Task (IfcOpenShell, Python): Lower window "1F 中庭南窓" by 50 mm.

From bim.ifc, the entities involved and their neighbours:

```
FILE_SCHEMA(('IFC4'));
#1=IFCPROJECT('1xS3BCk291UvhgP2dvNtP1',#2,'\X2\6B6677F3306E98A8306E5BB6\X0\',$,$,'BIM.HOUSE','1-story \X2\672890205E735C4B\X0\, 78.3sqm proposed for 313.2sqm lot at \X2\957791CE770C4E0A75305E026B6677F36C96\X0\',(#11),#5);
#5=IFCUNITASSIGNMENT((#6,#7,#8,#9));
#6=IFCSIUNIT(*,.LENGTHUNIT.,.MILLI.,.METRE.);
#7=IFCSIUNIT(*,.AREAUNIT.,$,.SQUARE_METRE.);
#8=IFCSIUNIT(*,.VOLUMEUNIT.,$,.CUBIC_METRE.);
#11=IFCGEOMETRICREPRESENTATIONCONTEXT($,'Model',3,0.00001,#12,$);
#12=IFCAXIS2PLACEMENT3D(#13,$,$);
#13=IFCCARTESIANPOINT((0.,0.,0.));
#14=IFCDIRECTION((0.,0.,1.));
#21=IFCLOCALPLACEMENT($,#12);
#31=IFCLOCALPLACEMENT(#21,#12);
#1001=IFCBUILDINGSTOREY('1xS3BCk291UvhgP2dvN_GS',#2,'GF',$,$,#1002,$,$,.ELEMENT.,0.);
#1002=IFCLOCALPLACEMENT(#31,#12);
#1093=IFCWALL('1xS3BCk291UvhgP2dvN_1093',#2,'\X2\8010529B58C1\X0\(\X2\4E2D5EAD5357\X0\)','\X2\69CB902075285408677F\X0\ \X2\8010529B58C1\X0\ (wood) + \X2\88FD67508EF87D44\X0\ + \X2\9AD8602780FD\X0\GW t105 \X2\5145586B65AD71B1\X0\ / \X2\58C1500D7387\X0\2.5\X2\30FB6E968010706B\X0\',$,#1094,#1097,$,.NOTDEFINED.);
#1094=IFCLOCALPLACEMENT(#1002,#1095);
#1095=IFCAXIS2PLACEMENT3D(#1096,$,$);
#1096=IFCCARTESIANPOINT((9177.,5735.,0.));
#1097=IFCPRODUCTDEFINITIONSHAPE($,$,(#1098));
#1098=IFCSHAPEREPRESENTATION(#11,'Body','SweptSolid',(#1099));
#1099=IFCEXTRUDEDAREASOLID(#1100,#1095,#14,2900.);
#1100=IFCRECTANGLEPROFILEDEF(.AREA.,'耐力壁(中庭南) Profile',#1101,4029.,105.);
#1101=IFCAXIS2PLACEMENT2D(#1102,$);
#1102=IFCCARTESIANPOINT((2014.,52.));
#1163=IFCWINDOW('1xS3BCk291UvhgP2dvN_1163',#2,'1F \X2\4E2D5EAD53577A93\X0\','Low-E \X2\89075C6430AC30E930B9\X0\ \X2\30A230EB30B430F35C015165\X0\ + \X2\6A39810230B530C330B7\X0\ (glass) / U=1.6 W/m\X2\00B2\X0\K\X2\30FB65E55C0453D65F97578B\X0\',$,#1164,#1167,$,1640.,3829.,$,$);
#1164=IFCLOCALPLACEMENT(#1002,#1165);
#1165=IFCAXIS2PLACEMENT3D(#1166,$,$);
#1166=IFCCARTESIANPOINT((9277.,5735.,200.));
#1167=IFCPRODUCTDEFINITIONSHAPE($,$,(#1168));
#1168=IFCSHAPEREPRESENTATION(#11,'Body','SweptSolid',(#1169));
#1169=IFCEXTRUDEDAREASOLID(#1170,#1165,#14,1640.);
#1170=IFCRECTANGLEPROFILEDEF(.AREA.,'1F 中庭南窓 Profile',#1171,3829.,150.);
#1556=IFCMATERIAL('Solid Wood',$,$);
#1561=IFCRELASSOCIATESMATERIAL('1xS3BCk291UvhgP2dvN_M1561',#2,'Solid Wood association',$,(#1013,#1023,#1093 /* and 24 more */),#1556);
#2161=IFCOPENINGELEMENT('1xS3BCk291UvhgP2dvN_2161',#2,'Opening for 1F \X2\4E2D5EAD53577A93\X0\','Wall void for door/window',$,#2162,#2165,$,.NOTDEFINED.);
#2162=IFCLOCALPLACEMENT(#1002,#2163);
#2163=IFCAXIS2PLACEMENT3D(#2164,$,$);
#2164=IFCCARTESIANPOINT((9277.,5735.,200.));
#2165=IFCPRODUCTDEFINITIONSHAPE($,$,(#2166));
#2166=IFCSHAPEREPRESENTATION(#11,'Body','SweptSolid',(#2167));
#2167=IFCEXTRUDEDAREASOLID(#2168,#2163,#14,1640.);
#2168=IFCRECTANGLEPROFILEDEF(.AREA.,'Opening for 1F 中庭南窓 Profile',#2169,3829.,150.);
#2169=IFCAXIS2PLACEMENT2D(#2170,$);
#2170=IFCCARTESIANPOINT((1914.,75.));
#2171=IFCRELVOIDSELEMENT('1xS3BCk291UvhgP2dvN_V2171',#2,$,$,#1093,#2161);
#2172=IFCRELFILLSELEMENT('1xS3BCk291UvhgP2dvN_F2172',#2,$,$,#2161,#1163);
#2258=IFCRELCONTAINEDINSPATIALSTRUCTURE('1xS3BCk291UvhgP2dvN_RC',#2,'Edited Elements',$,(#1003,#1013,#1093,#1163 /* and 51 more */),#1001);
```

```python
import numpy as np
import ifcopenshell
import ifcopenshell.api.geometry
import ifcopenshell.util.placement
import ifcopenshell.util.unit

model = ifcopenshell.open("bim.ifc")
unit_scale = ifcopenshell.util.unit.calculate_unit_scale(model)

window = model.by_id(1163)
opening = window.FillsVoids[0].RelatingOpeningElement
dz = -50.0

shift = np.array([0.0, 0.0, dz])
# The window is not placed relative to its opening, so move both.
for product in (opening, window):
    matrix = ifcopenshell.util.placement.get_local_placement(product.ObjectPlacement)
    matrix[:3, 3] += shift
    ifcopenshell.api.geometry.edit_object_placement(model, product=product, matrix=matrix, is_si=False)

print(f"moved by {dz * unit_scale:+.3f} m")

model.write("bim_rev.ifc")
```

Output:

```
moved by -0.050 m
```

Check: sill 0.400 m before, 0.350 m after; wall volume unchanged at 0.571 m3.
